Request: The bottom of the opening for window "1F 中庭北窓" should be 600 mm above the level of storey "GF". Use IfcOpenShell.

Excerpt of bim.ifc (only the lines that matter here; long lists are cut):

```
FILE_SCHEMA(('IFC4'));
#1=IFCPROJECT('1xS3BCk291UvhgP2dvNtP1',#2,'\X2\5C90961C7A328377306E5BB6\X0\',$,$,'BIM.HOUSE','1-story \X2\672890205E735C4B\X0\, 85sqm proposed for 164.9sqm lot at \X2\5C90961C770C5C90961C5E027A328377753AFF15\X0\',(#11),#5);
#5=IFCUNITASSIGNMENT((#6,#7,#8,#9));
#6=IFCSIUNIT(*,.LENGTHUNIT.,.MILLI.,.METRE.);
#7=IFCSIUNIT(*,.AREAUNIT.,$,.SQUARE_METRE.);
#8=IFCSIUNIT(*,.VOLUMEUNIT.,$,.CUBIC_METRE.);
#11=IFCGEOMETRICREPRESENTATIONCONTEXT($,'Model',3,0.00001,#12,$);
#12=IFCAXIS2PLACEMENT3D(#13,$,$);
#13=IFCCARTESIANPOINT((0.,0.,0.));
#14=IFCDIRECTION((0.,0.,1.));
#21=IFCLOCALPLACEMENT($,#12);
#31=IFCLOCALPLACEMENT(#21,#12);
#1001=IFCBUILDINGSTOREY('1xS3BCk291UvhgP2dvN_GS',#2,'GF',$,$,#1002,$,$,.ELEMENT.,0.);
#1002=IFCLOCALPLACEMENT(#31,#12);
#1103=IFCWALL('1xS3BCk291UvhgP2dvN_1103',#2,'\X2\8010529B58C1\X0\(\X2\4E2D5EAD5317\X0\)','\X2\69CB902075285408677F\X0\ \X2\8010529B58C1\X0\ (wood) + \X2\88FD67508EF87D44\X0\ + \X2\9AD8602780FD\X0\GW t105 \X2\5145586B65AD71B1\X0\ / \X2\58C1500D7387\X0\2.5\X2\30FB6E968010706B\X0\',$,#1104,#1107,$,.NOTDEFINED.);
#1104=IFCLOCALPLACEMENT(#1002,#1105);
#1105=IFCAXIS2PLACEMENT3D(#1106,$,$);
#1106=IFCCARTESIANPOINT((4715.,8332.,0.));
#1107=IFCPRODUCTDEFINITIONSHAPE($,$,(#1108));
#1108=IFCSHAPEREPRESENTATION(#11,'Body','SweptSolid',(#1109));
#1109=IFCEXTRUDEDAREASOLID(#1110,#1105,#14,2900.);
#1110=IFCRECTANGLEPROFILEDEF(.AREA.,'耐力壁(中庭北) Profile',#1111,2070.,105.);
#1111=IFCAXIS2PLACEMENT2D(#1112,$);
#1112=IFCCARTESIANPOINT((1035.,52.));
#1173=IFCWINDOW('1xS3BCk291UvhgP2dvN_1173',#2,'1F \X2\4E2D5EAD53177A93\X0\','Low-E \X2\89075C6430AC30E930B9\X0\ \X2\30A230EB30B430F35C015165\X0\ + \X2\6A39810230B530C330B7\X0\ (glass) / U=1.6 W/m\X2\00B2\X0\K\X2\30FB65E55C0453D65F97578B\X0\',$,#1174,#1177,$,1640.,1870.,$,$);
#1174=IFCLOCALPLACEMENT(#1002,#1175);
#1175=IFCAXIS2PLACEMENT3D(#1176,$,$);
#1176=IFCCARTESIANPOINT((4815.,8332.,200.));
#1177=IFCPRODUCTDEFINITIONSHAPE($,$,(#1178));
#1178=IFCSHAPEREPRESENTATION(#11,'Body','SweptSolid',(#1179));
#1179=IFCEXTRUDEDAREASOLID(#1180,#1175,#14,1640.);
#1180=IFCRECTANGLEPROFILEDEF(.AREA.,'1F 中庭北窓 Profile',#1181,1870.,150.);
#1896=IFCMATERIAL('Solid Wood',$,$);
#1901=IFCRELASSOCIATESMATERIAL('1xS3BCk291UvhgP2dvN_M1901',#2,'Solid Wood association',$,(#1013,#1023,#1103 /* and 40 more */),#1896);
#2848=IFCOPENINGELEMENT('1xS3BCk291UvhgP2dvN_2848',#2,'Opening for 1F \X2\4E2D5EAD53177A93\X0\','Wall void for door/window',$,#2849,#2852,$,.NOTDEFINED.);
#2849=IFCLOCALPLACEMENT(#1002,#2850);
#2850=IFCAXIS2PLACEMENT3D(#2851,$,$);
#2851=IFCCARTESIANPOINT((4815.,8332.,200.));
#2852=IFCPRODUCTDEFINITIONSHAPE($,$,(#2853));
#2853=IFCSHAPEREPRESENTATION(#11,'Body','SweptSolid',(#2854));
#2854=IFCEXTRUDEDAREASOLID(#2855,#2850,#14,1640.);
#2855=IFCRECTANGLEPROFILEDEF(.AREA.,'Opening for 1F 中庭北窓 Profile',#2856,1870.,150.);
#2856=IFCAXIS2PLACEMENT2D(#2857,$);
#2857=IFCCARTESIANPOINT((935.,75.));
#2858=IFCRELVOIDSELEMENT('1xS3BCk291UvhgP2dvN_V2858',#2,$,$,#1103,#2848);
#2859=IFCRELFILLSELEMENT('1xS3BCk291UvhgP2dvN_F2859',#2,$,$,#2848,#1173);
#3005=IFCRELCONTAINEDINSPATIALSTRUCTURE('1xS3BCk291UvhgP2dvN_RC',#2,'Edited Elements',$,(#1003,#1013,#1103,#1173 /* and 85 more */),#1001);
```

```python
import numpy as np
import ifcopenshell
import ifcopenshell.api.geometry
import ifcopenshell.geom
import ifcopenshell.util.element
import ifcopenshell.util.placement
import ifcopenshell.util.shape
import ifcopenshell.util.unit

model = ifcopenshell.open("bim.ifc")
unit_scale = ifcopenshell.util.unit.calculate_unit_scale(model)

window = model.by_guid("1xS3BCk291UvhgP2dvN_1173")
opening = window.FillsVoids[0].RelatingOpeningElement
storey = ifcopenshell.util.element.get_container(window, ifc_class="IfcBuildingStorey")
level = ifcopenshell.util.placement.get_local_placement(storey.ObjectPlacement)[2, 3]

# The opening's origin need not be at the sill, so measure its lowest point.
shape = ifcopenshell.geom.create_shape(ifcopenshell.geom.settings(), opening)
bottom = ifcopenshell.util.shape.get_shape_bottom_elevation(shape, shape.geometry) / unit_scale
dz = level + 0.6 / unit_scale - bottom

shift = np.array([0.0, 0.0, dz])
# The window is not placed relative to its opening, so move both.
for product in (opening, window):
    matrix = ifcopenshell.util.placement.get_local_placement(product.ObjectPlacement)
    matrix[:3, 3] += shift
    ifcopenshell.api.geometry.edit_object_placement(model, product=product, matrix=matrix, is_si=False)

print(f"moved by {dz * unit_scale:+.3f} m")

model.write("bim_rev.ifc")
```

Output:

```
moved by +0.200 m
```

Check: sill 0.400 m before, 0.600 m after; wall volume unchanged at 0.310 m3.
